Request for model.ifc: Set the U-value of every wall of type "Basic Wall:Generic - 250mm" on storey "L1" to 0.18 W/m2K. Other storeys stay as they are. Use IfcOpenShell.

First a look at what the model holds.

```python
import ifcopenshell
import ifcopenshell.util.element

model = ifcopenshell.open("model.ifc")
print(model.schema)
storey = next(s for s in model.by_type("IfcBuildingStorey") if s.Name == "L1")
walls = [e for e in ifcopenshell.util.element.get_decomposition(storey) if e.is_a("IfcWall")]
seen = {}
for e in walls:
    element_type = ifcopenshell.util.element.get_type(e)
    key = (element_type.Name if element_type != e and element_type else None, ifcopenshell.util.element.get_pset(e, "Pset_WallCommon", "ThermalTransmittance"))
    seen[key] = seen.get(key, 0) + 1
for (name, value), count in sorted(seen.items(), key=str):
    print(count, "x", name, "|", value)
```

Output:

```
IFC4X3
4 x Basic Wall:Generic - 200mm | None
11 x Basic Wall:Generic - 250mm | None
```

```python
import ifcopenshell
import ifcopenshell.api.pset
import ifcopenshell.util.element

model = ifcopenshell.open("model.ifc")

storey = next(s for s in model.by_type("IfcBuildingStorey") if s.Name == "L1")
walls = [e for e in ifcopenshell.util.element.get_decomposition(storey) if e.is_a("IfcWall")]

count = 0
for e in walls:
    element_type = ifcopenshell.util.element.get_type(e)
    if element_type in (None, e) or element_type.Name != "Basic Wall:Generic - 250mm":
        continue
    # add_pset returns the element's existing set when there is one.
    pset = ifcopenshell.api.pset.add_pset(model, product=e, name="Pset_WallCommon")
    ifcopenshell.api.pset.edit_pset(model, pset=pset, properties={"ThermalTransmittance": 0.18})
    count += 1

print(count, "walls updated")

model.write("model_edited.ifc")
```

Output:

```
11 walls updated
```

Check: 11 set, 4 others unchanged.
